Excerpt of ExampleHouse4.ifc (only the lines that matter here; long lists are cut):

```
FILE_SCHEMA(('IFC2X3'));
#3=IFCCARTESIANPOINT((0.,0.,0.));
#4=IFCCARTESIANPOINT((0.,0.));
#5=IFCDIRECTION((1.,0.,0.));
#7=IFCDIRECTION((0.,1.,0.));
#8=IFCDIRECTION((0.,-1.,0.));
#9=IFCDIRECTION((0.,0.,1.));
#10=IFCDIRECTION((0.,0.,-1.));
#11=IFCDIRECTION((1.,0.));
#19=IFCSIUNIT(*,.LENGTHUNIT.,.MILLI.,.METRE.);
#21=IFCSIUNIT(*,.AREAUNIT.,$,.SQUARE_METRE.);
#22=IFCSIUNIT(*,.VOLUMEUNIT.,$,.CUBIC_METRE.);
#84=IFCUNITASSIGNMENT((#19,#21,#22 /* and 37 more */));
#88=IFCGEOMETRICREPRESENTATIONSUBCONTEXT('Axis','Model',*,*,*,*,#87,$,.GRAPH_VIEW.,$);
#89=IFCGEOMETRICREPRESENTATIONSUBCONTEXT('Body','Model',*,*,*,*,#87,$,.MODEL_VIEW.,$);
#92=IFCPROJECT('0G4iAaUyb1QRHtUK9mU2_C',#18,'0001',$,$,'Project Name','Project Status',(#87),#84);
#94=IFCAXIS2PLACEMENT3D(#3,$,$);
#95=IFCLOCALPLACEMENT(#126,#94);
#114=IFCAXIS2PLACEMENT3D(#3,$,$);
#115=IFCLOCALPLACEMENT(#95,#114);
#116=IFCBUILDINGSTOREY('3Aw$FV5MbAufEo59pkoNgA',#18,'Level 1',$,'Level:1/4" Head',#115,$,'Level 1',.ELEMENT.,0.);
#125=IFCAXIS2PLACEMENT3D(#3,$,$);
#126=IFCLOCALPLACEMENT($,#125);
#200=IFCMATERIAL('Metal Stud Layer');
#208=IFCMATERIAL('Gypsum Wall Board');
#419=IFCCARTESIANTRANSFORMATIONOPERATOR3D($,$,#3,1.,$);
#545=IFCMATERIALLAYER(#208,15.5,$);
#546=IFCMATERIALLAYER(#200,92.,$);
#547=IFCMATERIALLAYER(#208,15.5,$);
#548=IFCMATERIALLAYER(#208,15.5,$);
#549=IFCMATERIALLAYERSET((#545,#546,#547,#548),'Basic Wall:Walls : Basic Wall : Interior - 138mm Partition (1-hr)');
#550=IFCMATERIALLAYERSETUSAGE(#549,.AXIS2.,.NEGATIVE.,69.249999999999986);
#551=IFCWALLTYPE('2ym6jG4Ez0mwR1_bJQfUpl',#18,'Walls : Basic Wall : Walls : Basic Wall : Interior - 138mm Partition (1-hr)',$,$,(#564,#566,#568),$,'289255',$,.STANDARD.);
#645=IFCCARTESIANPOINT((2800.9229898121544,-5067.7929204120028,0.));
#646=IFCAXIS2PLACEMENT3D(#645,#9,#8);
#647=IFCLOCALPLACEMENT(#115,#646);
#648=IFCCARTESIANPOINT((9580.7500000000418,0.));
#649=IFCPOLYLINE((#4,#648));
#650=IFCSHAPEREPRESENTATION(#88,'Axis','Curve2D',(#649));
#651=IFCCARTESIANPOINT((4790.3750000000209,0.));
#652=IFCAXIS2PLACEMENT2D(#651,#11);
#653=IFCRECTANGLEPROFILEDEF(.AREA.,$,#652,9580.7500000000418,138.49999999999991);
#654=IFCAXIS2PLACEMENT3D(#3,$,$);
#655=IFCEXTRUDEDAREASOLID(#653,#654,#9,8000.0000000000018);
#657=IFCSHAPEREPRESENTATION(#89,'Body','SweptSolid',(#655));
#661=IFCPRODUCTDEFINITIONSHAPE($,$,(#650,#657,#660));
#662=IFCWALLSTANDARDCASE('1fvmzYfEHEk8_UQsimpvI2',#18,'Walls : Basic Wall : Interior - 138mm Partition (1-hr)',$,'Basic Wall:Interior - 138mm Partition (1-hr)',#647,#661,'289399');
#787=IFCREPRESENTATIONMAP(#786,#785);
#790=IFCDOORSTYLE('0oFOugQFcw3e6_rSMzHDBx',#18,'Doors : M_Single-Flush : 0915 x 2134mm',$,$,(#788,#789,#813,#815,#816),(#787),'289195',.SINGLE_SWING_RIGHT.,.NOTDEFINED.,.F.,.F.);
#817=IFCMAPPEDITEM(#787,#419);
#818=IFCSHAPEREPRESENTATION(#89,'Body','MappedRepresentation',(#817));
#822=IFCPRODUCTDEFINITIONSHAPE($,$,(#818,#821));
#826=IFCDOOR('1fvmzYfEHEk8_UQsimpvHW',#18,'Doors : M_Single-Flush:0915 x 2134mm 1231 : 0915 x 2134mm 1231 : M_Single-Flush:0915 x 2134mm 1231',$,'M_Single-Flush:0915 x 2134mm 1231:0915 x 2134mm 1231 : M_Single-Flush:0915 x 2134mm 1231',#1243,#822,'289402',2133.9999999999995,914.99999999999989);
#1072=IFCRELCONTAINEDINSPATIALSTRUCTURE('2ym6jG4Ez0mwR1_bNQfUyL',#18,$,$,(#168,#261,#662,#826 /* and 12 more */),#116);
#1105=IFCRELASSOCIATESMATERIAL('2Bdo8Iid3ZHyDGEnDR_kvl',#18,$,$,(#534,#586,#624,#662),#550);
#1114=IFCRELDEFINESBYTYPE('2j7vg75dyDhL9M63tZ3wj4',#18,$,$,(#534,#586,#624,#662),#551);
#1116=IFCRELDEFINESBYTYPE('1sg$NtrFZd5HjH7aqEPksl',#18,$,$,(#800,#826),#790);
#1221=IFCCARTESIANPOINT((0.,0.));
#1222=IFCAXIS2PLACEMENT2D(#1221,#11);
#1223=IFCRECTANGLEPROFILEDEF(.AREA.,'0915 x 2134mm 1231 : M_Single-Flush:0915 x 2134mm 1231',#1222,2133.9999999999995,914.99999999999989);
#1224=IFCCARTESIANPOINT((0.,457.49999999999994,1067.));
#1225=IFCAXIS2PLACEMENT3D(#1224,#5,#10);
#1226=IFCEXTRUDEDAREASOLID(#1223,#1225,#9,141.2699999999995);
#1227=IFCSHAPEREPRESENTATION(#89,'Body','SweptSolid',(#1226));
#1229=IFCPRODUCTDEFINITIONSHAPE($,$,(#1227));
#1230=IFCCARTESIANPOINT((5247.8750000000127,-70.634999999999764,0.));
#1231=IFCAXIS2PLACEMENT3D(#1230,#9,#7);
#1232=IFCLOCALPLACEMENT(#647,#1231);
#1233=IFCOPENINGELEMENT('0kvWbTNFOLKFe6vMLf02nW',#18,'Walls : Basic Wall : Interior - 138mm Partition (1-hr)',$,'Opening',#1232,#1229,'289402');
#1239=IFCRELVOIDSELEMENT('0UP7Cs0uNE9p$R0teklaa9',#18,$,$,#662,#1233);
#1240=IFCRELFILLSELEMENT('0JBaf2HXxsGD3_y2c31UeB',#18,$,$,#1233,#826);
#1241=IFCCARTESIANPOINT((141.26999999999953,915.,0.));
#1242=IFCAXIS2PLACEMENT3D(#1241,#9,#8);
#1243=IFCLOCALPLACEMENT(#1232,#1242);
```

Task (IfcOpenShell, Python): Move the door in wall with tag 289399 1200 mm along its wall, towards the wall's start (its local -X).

```python
import ifcopenshell
import ifcopenshell.api.geometry
import ifcopenshell.util.placement

model = ifcopenshell.open("ExampleHouse4.ifc")

door = model.by_guid("1fvmzYfEHEk8_UQsimpvHW")
opening = door.FillsVoids[0].RelatingOpeningElement
wall = opening.VoidsElements[0].RelatingBuildingElement

wall_matrix = ifcopenshell.util.placement.get_local_placement(wall.ObjectPlacement)
shift = wall_matrix[:3, 0] * -1200.0
before = ifcopenshell.util.placement.get_local_placement(door.ObjectPlacement)[:3, 3].copy()

# The door is placed relative to its opening, so it follows when the opening moves.
matrix = ifcopenshell.util.placement.get_local_placement(opening.ObjectPlacement)
matrix[:3, 3] += shift
ifcopenshell.api.geometry.edit_object_placement(
    model, product=opening, matrix=matrix, is_si=False, should_transform_children=True
)

after = ifcopenshell.util.placement.get_local_placement(door.ObjectPlacement)[:3, 3]
print("door moved by", (after - before).round(3) + 0.0)

model.write("ExampleHouse4_v2.ifc")
```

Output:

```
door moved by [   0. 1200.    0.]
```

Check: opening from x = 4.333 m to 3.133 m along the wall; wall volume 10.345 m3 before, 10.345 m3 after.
